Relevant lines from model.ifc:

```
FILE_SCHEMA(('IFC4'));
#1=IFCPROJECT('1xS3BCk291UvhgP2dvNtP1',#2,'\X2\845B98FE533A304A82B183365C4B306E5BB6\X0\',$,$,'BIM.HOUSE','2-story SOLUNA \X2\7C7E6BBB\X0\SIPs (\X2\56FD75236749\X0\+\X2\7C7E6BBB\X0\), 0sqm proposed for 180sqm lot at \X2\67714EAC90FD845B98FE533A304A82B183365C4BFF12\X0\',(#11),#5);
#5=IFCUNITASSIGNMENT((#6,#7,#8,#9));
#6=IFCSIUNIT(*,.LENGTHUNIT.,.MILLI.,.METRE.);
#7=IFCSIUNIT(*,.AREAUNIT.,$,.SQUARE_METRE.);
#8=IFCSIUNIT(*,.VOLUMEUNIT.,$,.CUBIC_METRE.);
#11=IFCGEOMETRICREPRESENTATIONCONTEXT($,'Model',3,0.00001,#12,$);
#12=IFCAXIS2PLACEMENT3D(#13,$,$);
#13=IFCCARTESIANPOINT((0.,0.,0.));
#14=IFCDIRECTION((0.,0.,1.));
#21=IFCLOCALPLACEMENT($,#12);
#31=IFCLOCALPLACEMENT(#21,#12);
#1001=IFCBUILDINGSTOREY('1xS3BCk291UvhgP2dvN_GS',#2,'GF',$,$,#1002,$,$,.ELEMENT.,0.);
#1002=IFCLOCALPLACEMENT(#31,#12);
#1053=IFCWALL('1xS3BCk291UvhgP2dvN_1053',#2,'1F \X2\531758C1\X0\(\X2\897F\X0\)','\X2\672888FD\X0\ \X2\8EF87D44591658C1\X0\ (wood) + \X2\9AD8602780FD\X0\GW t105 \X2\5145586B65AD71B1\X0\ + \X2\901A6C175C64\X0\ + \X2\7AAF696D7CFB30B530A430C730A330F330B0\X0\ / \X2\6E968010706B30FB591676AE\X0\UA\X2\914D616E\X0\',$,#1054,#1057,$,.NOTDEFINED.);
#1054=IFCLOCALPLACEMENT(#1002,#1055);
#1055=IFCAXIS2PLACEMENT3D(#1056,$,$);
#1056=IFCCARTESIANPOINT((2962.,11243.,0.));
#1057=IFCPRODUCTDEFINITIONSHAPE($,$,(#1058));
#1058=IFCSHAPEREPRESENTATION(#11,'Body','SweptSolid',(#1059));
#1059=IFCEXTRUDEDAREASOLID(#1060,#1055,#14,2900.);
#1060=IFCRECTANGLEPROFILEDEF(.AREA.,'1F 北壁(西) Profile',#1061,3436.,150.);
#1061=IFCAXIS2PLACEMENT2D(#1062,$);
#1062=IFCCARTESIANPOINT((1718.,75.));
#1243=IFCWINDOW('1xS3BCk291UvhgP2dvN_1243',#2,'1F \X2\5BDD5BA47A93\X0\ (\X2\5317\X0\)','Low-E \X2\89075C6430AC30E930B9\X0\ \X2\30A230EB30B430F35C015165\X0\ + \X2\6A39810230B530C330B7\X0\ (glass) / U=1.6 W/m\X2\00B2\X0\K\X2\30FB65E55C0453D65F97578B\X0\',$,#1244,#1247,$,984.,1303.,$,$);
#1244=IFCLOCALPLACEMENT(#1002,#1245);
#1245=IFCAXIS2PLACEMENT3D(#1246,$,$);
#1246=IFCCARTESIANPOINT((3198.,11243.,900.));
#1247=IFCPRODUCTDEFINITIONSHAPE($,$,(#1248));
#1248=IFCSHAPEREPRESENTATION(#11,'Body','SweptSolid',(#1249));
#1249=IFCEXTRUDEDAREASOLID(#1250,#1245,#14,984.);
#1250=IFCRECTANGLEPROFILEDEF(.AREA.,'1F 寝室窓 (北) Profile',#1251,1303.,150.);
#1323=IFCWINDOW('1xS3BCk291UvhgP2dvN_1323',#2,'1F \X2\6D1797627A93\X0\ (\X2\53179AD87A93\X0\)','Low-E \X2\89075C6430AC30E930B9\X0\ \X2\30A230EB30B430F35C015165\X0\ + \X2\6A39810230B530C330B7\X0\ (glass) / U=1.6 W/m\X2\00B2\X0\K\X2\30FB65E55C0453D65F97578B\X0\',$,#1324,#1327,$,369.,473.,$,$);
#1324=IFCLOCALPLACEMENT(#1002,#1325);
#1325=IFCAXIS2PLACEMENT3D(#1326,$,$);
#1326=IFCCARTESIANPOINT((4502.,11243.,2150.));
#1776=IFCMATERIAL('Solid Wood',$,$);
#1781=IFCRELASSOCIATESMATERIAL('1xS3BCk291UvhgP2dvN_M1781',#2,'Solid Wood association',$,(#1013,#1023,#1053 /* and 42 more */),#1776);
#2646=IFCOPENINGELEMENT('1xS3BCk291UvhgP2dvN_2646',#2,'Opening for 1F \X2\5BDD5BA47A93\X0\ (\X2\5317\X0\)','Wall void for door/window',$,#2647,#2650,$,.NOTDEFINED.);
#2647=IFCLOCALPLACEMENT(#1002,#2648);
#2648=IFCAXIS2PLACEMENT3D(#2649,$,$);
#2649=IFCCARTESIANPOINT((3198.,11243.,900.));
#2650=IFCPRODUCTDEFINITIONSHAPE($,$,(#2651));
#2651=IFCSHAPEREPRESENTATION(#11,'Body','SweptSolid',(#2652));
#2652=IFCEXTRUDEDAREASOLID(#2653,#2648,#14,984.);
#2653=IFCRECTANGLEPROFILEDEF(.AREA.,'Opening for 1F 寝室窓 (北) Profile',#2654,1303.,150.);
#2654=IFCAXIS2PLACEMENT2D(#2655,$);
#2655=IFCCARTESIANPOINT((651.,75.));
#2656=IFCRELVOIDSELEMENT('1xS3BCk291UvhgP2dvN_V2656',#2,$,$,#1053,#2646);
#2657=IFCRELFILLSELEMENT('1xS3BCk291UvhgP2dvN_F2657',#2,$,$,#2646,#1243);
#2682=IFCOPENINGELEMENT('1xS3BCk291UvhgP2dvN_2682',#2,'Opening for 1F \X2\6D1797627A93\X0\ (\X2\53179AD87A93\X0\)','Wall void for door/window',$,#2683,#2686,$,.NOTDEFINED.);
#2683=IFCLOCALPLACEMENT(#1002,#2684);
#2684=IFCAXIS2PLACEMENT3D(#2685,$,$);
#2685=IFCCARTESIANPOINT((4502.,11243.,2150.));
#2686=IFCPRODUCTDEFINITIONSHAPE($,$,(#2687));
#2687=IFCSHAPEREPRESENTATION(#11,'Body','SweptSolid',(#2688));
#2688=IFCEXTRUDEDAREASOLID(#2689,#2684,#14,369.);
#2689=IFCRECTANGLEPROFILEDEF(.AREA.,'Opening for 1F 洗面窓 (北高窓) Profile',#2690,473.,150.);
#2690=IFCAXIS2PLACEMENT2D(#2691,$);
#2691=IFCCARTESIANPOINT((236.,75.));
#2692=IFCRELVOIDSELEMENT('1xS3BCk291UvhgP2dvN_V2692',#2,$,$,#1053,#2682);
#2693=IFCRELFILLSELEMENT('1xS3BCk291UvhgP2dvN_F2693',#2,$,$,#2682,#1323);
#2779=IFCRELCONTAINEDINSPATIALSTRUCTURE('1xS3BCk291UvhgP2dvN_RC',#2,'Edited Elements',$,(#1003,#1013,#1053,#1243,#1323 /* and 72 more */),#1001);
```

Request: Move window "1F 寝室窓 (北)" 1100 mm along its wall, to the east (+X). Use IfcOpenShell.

```python
import ifcopenshell
import ifcopenshell.api.geometry
import ifcopenshell.util.placement

model = ifcopenshell.open("model.ifc")

window = model.by_guid("1xS3BCk291UvhgP2dvN_1243")
opening = window.FillsVoids[0].RelatingOpeningElement
wall = opening.VoidsElements[0].RelatingBuildingElement

wall_matrix = ifcopenshell.util.placement.get_local_placement(wall.ObjectPlacement)
shift = wall_matrix[:3, 0] * 1100.0
before = ifcopenshell.util.placement.get_local_placement(window.ObjectPlacement)[:3, 3].copy()

# The window is not placed relative to its opening, so move both.
for product in (opening, window):
    matrix = ifcopenshell.util.placement.get_local_placement(product.ObjectPlacement)
    matrix[:3, 3] += shift
    ifcopenshell.api.geometry.edit_object_placement(model, product=product, matrix=matrix, is_si=False)

after = ifcopenshell.util.placement.get_local_placement(window.ObjectPlacement)[:3, 3]
print("window moved by", (after - before).round(3) + 0.0)

model.write("model_updated.ifc")
```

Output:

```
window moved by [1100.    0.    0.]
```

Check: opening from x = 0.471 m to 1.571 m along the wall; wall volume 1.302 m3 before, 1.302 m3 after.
